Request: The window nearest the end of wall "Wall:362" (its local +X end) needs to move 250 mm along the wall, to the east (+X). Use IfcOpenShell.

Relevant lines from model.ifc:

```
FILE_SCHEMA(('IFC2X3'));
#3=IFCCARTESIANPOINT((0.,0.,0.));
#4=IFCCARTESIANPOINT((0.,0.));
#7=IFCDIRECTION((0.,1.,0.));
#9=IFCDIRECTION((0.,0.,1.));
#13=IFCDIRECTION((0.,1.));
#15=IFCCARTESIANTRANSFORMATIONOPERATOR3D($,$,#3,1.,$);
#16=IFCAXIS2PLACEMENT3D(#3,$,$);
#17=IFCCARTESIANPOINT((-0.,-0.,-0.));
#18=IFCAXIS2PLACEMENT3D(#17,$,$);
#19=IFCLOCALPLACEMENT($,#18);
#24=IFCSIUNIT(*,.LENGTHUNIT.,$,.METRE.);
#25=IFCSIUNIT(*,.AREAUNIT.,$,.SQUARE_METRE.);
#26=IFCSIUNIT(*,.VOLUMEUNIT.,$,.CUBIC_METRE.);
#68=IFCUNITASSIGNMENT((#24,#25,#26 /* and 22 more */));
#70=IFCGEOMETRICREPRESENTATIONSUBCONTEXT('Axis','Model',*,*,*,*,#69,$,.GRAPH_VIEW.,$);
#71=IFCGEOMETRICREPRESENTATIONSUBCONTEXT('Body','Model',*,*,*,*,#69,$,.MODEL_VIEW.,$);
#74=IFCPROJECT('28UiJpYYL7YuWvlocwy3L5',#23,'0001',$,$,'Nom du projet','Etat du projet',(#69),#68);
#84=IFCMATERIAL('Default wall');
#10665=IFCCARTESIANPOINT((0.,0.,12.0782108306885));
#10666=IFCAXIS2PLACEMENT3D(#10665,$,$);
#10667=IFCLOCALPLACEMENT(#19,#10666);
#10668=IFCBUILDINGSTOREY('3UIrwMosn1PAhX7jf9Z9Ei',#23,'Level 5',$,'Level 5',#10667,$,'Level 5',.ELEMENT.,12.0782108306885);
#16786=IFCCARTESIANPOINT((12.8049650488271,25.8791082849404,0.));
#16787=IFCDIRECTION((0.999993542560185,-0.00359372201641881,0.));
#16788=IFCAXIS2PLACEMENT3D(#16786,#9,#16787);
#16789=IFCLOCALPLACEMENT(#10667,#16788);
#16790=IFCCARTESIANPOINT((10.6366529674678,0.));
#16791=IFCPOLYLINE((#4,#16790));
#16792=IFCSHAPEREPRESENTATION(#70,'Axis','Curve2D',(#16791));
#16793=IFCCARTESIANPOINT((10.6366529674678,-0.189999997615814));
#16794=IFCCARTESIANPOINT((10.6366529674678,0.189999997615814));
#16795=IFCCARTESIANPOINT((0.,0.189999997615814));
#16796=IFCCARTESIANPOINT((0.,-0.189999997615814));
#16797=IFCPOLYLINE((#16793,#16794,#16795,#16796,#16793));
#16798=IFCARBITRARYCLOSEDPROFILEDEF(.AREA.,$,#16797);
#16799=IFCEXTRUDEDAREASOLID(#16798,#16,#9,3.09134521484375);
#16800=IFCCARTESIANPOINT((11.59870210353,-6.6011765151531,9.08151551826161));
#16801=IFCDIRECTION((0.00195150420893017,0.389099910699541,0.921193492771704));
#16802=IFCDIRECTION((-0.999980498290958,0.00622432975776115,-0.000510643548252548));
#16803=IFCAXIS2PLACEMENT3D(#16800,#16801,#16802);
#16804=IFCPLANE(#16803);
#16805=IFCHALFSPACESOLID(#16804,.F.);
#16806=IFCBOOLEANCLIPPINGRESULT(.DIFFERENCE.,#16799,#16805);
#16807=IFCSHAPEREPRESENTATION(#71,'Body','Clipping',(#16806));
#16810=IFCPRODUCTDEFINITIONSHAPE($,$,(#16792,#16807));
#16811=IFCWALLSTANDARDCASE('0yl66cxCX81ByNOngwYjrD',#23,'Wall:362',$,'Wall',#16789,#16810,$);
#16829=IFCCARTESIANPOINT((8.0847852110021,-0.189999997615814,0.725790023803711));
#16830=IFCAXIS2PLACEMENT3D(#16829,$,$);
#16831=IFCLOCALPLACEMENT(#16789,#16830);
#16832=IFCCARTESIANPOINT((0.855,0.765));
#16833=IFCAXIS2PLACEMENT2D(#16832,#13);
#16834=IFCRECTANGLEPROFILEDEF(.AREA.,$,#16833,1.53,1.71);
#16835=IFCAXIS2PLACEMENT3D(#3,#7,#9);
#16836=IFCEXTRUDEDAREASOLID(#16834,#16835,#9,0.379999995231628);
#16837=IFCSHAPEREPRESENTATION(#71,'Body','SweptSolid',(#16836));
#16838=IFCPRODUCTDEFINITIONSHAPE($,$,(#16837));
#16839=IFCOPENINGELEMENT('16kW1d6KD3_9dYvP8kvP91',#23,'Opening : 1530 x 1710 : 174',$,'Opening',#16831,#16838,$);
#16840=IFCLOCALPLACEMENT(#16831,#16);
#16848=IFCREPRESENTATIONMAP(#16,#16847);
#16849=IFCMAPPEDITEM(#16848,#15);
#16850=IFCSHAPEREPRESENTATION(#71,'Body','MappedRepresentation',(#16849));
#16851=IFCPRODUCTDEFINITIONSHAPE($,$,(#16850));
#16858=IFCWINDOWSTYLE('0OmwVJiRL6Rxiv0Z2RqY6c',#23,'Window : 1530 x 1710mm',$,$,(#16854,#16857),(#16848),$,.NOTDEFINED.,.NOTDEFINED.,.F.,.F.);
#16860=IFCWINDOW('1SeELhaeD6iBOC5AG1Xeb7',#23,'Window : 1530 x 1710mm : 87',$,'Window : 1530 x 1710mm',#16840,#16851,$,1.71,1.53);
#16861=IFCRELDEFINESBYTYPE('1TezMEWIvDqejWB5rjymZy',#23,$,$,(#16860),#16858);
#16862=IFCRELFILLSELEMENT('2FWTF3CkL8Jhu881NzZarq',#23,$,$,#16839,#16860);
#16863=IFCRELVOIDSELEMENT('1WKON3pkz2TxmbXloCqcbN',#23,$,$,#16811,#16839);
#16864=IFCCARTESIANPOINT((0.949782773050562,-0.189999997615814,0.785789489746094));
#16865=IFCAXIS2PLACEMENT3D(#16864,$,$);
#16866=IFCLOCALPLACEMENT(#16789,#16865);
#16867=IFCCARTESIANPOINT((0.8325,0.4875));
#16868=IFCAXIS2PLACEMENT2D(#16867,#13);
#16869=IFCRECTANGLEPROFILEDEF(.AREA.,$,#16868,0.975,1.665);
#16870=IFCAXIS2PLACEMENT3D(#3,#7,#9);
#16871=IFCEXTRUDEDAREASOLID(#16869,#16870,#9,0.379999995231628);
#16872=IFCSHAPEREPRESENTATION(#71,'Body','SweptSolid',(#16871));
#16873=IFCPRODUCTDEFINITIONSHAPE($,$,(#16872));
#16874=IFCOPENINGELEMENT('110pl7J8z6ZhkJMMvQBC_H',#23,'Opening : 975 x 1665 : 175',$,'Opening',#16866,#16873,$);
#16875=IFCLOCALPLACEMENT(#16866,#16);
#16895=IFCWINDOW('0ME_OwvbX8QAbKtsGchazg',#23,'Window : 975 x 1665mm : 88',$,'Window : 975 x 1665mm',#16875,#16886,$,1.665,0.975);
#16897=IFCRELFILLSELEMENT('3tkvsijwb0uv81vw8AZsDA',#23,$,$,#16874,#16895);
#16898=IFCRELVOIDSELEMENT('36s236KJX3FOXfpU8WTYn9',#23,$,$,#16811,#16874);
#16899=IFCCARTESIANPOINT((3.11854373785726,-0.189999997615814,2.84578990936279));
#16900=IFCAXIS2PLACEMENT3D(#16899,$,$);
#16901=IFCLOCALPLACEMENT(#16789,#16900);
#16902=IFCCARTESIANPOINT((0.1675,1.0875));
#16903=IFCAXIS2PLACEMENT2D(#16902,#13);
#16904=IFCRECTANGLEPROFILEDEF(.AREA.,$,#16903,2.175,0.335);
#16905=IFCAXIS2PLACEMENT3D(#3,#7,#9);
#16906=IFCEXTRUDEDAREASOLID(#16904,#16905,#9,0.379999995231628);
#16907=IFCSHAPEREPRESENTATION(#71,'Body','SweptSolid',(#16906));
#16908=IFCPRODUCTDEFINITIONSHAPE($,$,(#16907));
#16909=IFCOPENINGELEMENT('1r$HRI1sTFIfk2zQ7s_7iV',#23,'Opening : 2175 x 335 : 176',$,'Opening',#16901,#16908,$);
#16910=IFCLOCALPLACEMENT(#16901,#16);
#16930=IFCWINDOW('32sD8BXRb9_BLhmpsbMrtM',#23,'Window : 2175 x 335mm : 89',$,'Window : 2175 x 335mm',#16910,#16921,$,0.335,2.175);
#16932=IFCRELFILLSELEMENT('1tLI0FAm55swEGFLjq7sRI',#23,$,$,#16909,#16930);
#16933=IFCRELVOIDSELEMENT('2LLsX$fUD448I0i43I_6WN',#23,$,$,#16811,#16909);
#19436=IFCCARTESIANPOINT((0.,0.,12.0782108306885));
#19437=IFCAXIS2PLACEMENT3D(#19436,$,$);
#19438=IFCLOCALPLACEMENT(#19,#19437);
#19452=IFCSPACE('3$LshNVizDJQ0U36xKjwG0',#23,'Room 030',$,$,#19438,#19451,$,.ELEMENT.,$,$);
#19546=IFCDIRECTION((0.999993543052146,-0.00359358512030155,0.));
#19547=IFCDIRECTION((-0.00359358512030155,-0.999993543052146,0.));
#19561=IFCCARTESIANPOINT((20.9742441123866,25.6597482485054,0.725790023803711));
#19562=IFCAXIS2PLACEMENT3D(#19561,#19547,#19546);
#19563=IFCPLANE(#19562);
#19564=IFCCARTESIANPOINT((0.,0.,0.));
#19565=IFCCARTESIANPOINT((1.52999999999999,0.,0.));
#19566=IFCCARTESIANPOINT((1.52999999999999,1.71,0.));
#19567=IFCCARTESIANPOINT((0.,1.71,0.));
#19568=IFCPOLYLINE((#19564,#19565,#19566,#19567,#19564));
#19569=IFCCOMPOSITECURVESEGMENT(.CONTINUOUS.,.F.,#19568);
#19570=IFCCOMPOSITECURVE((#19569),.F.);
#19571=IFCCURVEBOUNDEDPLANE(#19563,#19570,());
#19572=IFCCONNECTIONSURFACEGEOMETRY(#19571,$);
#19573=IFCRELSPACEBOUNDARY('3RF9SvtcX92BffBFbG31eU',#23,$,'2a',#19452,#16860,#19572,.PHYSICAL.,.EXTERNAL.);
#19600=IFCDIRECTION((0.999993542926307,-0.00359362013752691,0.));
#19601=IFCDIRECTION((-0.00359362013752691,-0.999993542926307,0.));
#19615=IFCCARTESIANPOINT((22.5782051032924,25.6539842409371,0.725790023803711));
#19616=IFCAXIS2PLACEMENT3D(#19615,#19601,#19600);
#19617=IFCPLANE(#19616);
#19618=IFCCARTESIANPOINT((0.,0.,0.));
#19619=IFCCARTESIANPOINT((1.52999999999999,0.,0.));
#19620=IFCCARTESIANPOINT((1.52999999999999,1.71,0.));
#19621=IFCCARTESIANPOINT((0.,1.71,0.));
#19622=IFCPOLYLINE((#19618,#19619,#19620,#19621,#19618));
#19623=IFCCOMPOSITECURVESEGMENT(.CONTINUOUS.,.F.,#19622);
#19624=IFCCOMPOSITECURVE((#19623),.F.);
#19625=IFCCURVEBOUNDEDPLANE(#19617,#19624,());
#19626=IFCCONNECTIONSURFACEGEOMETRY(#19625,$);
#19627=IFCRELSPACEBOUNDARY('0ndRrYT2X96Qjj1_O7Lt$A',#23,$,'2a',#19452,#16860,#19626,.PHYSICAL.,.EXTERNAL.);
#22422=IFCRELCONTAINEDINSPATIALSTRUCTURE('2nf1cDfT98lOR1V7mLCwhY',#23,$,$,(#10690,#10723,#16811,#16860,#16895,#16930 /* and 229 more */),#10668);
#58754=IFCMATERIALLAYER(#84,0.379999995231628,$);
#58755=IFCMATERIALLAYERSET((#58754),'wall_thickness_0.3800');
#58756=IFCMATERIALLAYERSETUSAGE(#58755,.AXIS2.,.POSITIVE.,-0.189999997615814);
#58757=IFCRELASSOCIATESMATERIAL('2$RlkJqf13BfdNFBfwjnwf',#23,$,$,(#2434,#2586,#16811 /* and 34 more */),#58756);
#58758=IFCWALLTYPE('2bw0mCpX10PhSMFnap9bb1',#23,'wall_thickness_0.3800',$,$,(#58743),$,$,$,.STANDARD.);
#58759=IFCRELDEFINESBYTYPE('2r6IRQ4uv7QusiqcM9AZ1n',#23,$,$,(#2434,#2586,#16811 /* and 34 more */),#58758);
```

```python
import numpy as np
import ifcopenshell
import ifcopenshell.api.geometry
import ifcopenshell.util.placement
import ifcopenshell.util.unit

model = ifcopenshell.open("model.ifc")
unit_scale = ifcopenshell.util.unit.calculate_unit_scale(model)

window = model.by_guid("1SeELhaeD6iBOC5AG1Xeb7")
opening = window.FillsVoids[0].RelatingOpeningElement
wall = opening.VoidsElements[0].RelatingBuildingElement

wall_matrix = ifcopenshell.util.placement.get_local_placement(wall.ObjectPlacement)
shift = wall_matrix[:3, 0] * 0.25 / unit_scale
before = ifcopenshell.util.placement.get_local_placement(window.ObjectPlacement)[:3, 3].copy()

# The window is placed relative to its opening, so it follows when the opening moves.
matrix = ifcopenshell.util.placement.get_local_placement(opening.ObjectPlacement)
matrix[:3, 3] += shift
ifcopenshell.api.geometry.edit_object_placement(
    model, product=opening, matrix=matrix, is_si=False, should_transform_children=True
)

# Space boundary surfaces are stored in each space's coordinates; move them too.
for rel in window.ProvidesBoundaries:
    if not rel.ConnectionGeometry:
        continue
    surface = rel.ConnectionGeometry.SurfaceOnRelatingElement.BasisSurface
    space_matrix = ifcopenshell.util.placement.get_local_placement(rel.RelatingSpace.ObjectPlacement)
    point = np.array(surface.Position.Location.Coordinates) + space_matrix[:3, :3].T @ shift
    surface.Position = model.createIfcAxis2Placement3D(
        model.createIfcCartesianPoint(point.tolist()), surface.Position.Axis, surface.Position.RefDirection
    )

after = ifcopenshell.util.placement.get_local_placement(window.ObjectPlacement)[:3, 3]
print("window moved by", (after - before).round(3) + 0.0)

model.write("model_v2.ifc")
```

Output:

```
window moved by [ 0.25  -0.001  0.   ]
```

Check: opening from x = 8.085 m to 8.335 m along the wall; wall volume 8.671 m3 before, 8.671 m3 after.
